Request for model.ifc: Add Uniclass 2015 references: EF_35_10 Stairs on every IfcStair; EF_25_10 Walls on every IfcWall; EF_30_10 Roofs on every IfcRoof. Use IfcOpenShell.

First a look at what the model holds.

```python
import ifcopenshell

model = ifcopenshell.open("model.ifc")
print(model.schema)
print("classifications:", [c.Name for c in model.by_type("IfcClassification")])
for ifc_class in ("IfcDoor", "IfcRoof", "IfcStair", "IfcWall", "IfcWindow"):
    print(ifc_class, len(model.by_type(ifc_class)))
```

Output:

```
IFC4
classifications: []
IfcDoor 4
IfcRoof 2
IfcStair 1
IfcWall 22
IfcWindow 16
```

```python
import ifcopenshell
import ifcopenshell.api.classification

model = ifcopenshell.open("model.ifc")

system = ifcopenshell.api.classification.add_classification(model, classification="Uniclass 2015")

codes = {
    "IfcStair": ("EF_35_10", "Stairs"),
    "IfcWall": ("EF_25_10", "Walls"),
    "IfcRoof": ("EF_30_10", "Roofs"),
}
for ifc_class, (code, name) in codes.items():
    products = model.by_type(ifc_class)
    ifcopenshell.api.classification.add_reference(
        model, products=products, classification=system, identification=code, name=name
    )
    print(code, len(products))

model.write("model_rev.ifc")
```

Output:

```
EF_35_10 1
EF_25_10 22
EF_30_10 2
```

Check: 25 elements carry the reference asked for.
